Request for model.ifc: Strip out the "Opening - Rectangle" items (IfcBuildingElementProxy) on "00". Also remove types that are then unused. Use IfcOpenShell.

First a look at what the model holds.

```python
import ifcopenshell
import ifcopenshell.util.element

model = ifcopenshell.open("model.ifc")
print(model.schema)
storey = next(s for s in model.by_type("IfcBuildingStorey") if s.Name == "00")
proxies = [e for e in ifcopenshell.util.element.get_decomposition(storey) if e.is_a("IfcBuildingElementProxy")]
seen = {}
for e in proxies:
    element_type = ifcopenshell.util.element.get_type(e)
    name = element_type.Name if element_type not in (None, e) else None
    seen[name] = seen.get(name, 0) + 1
for name, count in sorted(seen.items(), key=str):
    print(count, "x", name)
```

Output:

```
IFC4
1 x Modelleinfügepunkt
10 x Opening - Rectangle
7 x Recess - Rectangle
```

```python
import ifcopenshell
import ifcopenshell.api.root
import ifcopenshell.util.element

model = ifcopenshell.open("model.ifc")

storey = next(s for s in model.by_type("IfcBuildingStorey") if s.Name == "00")
proxies = [e for e in ifcopenshell.util.element.get_decomposition(storey) if e.is_a("IfcBuildingElementProxy")]
targets = [e for e in proxies if (t := ifcopenshell.util.element.get_type(e)) not in (None, e) and t.Name == "Opening - Rectangle"]
types = {ifcopenshell.util.element.get_type(e) for e in targets} - {None, *targets}

for e in targets:
    ifcopenshell.api.root.remove_product(model, product=e)
print(len(targets), "removed")

unused = [t for t in types if not ifcopenshell.util.element.get_types(t)]
for t in unused:
    ifcopenshell.api.root.remove_product(model, product=t)
print(len(unused), "unused types removed")

model.write("model_rev.ifc")
```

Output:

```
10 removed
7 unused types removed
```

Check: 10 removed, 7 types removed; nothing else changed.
